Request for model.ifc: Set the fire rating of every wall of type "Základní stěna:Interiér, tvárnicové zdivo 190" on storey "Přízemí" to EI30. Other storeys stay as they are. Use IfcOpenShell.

First a look at what the model holds.

```python
import ifcopenshell
import ifcopenshell.util.element

model = ifcopenshell.open("model.ifc")
print(model.schema)
storey = next(s for s in model.by_type("IfcBuildingStorey") if s.Name == "Přízemí")
walls = [e for e in ifcopenshell.util.element.get_decomposition(storey) if e.is_a("IfcWall")]
seen = {}
for e in walls:
    element_type = ifcopenshell.util.element.get_type(e)
    key = (element_type.Name if element_type != e and element_type else None, ifcopenshell.util.element.get_pset(e, "Pset_WallCommon", "FireRating"))
    seen[key] = seen.get(key, 0) + 1
for (name, value), count in sorted(seen.items(), key=str):
    print(count, "x", name, "|", value)
```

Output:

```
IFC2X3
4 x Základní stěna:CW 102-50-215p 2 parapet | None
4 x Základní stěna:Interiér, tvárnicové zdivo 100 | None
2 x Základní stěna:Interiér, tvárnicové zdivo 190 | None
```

```python
import ifcopenshell
import ifcopenshell.api.pset
import ifcopenshell.util.element

model = ifcopenshell.open("model.ifc")

storey = next(s for s in model.by_type("IfcBuildingStorey") if s.Name == "Přízemí")
walls = [e for e in ifcopenshell.util.element.get_decomposition(storey) if e.is_a("IfcWall")]

count = 0
for e in walls:
    element_type = ifcopenshell.util.element.get_type(e)
    if element_type in (None, e) or element_type.Name != "Základní stěna:Interiér, tvárnicové zdivo 190":
        continue
    # add_pset returns the element's existing set when there is one.
    pset = ifcopenshell.api.pset.add_pset(model, product=e, name="Pset_WallCommon")
    ifcopenshell.api.pset.edit_pset(model, pset=pset, properties={"FireRating": "EI30"})
    count += 1

print(count, "walls updated")

model.write("model_rev.ifc")
```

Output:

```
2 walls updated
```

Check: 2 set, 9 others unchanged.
